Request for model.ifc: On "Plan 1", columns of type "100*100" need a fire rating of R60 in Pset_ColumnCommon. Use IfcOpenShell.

First a look at what the model holds.

```python
import ifcopenshell
import ifcopenshell.util.element

model = ifcopenshell.open("model.ifc")
print(model.schema)
storey = next(s for s in model.by_type("IfcBuildingStorey") if s.Name == "Plan 1")
columns = [e for e in ifcopenshell.util.element.get_decomposition(storey) if e.is_a("IfcColumn")]
seen = {}
for e in columns:
    element_type = ifcopenshell.util.element.get_type(e)
    key = (element_type.Name if element_type != e and element_type else None, ifcopenshell.util.element.get_pset(e, "Pset_ColumnCommon", "FireRating"))
    seen[key] = seen.get(key, 0) + 1
for (name, value), count in sorted(seen.items(), key=str):
    print(count, "x", name, "|", value)
```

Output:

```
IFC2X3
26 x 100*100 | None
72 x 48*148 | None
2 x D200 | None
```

```python
import ifcopenshell
import ifcopenshell.api.pset
import ifcopenshell.util.element

model = ifcopenshell.open("model.ifc")

storey = next(s for s in model.by_type("IfcBuildingStorey") if s.Name == "Plan 1")
columns = [e for e in ifcopenshell.util.element.get_decomposition(storey) if e.is_a("IfcColumn")]

count = 0
for e in columns:
    element_type = ifcopenshell.util.element.get_type(e)
    if element_type in (None, e) or element_type.Name != "100*100":
        continue
    found = ifcopenshell.util.element.get_pset(e, "Pset_ColumnCommon", should_inherit=False)
    if found:
        pset = model.by_id(found["id"])
        if len(ifcopenshell.util.element.get_elements_by_pset(pset)) > 1:
            pset = ifcopenshell.api.pset.unshare_pset(model, products=[e], pset=pset)[0]
    else:
        pset = ifcopenshell.api.pset.add_pset(model, product=e, name="Pset_ColumnCommon")
    ifcopenshell.api.pset.edit_pset(model, pset=pset, properties={"FireRating": "R60"})
    count += 1

print(count, "columns updated")

model.write("model_v2.ifc")
```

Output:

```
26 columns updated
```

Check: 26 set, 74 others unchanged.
